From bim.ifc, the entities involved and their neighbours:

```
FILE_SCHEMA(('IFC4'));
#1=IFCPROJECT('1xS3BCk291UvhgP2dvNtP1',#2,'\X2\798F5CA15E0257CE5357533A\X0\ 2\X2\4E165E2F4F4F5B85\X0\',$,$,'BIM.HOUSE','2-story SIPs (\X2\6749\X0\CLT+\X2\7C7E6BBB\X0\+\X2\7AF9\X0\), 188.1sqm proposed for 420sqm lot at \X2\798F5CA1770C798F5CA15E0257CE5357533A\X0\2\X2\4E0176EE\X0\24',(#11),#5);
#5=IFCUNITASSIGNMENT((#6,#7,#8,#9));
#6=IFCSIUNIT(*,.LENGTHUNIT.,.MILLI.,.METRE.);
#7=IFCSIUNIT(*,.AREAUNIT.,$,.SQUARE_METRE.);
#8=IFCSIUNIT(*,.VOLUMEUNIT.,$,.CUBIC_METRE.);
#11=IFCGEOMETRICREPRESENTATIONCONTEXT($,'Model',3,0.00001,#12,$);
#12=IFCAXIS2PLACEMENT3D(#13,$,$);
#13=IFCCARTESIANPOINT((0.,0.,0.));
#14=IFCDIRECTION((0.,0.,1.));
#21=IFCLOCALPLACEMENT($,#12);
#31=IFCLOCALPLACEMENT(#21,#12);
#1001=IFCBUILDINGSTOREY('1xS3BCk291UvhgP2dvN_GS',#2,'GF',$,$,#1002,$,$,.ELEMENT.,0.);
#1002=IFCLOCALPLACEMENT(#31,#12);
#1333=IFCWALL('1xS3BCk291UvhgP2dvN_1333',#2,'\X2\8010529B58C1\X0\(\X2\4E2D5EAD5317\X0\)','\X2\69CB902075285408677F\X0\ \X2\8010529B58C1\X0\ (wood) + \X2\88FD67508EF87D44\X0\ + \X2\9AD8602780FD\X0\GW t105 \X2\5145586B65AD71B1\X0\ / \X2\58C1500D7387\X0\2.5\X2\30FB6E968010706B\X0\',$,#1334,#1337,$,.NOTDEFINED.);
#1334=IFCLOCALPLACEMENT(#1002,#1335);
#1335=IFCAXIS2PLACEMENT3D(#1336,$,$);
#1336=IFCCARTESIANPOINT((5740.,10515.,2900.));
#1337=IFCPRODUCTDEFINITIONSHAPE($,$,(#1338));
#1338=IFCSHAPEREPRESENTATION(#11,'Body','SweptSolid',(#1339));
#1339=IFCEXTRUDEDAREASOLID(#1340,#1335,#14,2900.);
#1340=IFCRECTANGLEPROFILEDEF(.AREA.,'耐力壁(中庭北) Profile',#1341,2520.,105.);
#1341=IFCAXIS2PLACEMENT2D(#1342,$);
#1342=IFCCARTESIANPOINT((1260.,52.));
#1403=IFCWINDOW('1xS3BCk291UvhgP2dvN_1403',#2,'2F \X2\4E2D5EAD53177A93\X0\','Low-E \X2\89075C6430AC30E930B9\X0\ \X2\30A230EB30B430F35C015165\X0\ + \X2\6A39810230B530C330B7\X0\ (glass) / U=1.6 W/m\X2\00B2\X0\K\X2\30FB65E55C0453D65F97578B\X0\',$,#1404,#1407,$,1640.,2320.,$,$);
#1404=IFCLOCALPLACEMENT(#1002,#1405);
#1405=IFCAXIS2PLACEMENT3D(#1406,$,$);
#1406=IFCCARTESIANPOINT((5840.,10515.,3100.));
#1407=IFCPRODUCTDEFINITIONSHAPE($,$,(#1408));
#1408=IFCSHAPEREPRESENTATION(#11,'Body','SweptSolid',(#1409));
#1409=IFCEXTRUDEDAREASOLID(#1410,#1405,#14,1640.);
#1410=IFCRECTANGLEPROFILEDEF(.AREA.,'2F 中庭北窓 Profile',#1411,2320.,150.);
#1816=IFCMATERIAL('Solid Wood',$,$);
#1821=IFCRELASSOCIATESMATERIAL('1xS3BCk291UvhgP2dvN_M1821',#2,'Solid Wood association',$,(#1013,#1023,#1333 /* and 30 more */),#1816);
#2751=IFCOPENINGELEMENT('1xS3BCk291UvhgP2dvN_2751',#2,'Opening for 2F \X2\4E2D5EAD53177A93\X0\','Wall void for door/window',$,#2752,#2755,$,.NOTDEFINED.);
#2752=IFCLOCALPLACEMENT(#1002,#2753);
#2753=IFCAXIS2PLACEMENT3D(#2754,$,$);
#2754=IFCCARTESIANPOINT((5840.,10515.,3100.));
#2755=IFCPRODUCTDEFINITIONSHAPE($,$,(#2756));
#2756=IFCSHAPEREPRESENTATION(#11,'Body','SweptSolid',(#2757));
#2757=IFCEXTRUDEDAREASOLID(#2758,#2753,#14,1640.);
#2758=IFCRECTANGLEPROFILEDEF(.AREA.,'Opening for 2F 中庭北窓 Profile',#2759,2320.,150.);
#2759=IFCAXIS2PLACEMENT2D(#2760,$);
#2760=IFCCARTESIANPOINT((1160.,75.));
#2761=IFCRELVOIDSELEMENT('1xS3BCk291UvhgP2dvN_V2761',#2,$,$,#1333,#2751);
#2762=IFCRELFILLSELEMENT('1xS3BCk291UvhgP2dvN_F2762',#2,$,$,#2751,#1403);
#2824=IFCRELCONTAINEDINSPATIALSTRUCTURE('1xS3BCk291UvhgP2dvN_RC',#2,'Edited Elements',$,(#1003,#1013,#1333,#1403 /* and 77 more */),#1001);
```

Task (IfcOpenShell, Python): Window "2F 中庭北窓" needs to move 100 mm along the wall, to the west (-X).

```python
import ifcopenshell
import ifcopenshell.api.geometry
import ifcopenshell.util.placement
import ifcopenshell.util.unit

model = ifcopenshell.open("bim.ifc")
unit_scale = ifcopenshell.util.unit.calculate_unit_scale(model)

window = model.by_guid("1xS3BCk291UvhgP2dvN_1403")
opening = window.FillsVoids[0].RelatingOpeningElement
wall = opening.VoidsElements[0].RelatingBuildingElement

wall_matrix = ifcopenshell.util.placement.get_local_placement(wall.ObjectPlacement)
shift = wall_matrix[:3, 0] * -0.1 / unit_scale
before = ifcopenshell.util.placement.get_local_placement(window.ObjectPlacement)[:3, 3].copy()

# The window is not placed relative to its opening, so move both.
for product in (opening, window):
    matrix = ifcopenshell.util.placement.get_local_placement(product.ObjectPlacement)
    matrix[:3, 3] += shift
    ifcopenshell.api.geometry.edit_object_placement(model, product=product, matrix=matrix, is_si=False)

after = ifcopenshell.util.placement.get_local_placement(window.ObjectPlacement)[:3, 3]
print("window moved by", (after - before).round(3) + 0.0)

model.write("bim_updated.ifc")
```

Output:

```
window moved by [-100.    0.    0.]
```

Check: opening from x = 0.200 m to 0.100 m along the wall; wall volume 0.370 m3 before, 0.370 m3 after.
